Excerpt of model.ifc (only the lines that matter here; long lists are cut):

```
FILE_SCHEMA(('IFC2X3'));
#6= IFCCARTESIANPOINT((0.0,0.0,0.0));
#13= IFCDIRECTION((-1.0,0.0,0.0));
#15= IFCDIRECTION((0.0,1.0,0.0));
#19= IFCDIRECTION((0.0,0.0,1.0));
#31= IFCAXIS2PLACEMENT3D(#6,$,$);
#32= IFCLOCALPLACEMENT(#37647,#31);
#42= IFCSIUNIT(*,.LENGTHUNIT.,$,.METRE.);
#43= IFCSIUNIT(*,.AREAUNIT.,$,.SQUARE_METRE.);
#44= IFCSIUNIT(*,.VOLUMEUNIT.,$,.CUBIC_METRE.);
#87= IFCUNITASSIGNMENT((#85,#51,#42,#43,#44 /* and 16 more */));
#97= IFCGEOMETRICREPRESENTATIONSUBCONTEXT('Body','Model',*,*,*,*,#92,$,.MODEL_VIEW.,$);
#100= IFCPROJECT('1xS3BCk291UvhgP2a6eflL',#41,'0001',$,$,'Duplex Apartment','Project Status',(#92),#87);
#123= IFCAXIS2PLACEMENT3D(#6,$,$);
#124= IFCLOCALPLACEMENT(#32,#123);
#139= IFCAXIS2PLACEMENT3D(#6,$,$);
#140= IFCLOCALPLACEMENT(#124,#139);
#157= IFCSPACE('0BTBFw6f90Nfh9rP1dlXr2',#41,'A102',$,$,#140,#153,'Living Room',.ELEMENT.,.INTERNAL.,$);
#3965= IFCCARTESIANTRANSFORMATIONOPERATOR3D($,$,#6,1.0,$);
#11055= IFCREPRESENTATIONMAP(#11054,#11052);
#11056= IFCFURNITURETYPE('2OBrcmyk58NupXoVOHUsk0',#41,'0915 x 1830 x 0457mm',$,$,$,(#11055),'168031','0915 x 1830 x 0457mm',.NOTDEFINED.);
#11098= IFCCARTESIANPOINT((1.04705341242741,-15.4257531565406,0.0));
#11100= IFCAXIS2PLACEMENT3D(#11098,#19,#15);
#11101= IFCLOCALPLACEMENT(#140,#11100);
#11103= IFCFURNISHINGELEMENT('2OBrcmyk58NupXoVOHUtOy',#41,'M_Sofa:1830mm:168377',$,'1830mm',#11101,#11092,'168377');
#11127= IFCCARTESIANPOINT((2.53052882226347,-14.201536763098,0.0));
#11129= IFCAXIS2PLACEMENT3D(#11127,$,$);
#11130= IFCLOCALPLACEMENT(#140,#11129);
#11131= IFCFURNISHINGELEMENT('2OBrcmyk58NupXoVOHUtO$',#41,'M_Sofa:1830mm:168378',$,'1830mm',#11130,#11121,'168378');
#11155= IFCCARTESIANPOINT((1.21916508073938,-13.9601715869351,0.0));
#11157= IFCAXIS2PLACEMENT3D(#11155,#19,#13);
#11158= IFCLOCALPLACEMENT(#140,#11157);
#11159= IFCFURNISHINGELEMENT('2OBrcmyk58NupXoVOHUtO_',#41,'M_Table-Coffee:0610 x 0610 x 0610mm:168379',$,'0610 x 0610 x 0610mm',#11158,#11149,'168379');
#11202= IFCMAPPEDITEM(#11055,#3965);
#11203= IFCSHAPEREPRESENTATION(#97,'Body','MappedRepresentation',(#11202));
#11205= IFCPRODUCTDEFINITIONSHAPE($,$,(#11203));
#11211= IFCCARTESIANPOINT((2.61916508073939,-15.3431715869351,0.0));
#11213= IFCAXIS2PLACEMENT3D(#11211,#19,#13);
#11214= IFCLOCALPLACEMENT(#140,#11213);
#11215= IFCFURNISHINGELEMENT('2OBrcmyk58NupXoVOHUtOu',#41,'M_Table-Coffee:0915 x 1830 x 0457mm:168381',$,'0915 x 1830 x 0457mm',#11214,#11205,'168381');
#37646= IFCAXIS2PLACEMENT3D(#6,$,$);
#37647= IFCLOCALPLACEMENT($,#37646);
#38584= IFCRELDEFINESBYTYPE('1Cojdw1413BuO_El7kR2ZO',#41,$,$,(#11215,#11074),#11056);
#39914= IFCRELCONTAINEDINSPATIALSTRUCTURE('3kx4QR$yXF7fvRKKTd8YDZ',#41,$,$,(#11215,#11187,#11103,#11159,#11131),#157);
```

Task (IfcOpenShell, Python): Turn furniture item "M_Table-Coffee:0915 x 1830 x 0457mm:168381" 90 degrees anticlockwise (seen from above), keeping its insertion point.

```python
import ifcopenshell
import ifcopenshell.api.geometry
import ifcopenshell.util.placement

model = ifcopenshell.open("model.ifc")

item = model.by_guid("2OBrcmyk58NupXoVOHUtOu")
matrix = ifcopenshell.util.placement.get_local_placement(item.ObjectPlacement)
matrix = matrix @ ifcopenshell.util.placement.rotation(90, "Z")
ifcopenshell.api.geometry.edit_object_placement(model, product=item, matrix=matrix, is_si=False)

print(ifcopenshell.util.placement.get_local_placement(item.ObjectPlacement).round(3) + 0.0)

model.write("model_edited.ifc")
```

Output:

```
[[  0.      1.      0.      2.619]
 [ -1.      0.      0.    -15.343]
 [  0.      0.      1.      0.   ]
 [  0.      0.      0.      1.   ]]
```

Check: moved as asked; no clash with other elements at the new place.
